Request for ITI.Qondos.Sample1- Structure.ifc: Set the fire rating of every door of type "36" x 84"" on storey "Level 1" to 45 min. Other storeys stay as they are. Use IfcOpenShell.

First a look at what the model holds.

```python
import ifcopenshell
import ifcopenshell.util.element

model = ifcopenshell.open("ITI.Qondos.Sample1- Structure.ifc")
print(model.schema)
storey = next(s for s in model.by_type("IfcBuildingStorey") if s.Name == "Level 1")
doors = [e for e in ifcopenshell.util.element.get_decomposition(storey) if e.is_a("IfcDoor")]
seen = {}
for e in doors:
    element_type = ifcopenshell.util.element.get_type(e)
    key = (element_type.Name if element_type != e and element_type else None, ifcopenshell.util.element.get_pset(e, "Pset_DoorCommon", "FireRating"))
    seen[key] = seen.get(key, 0) + 1
for (name, value), count in sorted(seen.items(), key=str):
    print(count, "x", name, "|", value)
```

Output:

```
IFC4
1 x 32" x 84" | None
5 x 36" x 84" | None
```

```python
import ifcopenshell
import ifcopenshell.api.pset
import ifcopenshell.util.element

model = ifcopenshell.open("ITI.Qondos.Sample1- Structure.ifc")

storey = next(s for s in model.by_type("IfcBuildingStorey") if s.Name == "Level 1")
doors = [e for e in ifcopenshell.util.element.get_decomposition(storey) if e.is_a("IfcDoor")]

count = 0
for e in doors:
    element_type = ifcopenshell.util.element.get_type(e)
    if element_type in (None, e) or element_type.Name != '36" x 84"':
        continue
    # add_pset returns the element's existing set when there is one.
    pset = ifcopenshell.api.pset.add_pset(model, product=e, name="Pset_DoorCommon")
    ifcopenshell.api.pset.edit_pset(model, pset=pset, properties={"FireRating": "45 min"})
    count += 1

print(count, "doors updated")

model.write("ITI.Qondos.Sample1- Structure_v2.ifc")
```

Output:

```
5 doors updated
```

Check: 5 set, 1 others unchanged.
